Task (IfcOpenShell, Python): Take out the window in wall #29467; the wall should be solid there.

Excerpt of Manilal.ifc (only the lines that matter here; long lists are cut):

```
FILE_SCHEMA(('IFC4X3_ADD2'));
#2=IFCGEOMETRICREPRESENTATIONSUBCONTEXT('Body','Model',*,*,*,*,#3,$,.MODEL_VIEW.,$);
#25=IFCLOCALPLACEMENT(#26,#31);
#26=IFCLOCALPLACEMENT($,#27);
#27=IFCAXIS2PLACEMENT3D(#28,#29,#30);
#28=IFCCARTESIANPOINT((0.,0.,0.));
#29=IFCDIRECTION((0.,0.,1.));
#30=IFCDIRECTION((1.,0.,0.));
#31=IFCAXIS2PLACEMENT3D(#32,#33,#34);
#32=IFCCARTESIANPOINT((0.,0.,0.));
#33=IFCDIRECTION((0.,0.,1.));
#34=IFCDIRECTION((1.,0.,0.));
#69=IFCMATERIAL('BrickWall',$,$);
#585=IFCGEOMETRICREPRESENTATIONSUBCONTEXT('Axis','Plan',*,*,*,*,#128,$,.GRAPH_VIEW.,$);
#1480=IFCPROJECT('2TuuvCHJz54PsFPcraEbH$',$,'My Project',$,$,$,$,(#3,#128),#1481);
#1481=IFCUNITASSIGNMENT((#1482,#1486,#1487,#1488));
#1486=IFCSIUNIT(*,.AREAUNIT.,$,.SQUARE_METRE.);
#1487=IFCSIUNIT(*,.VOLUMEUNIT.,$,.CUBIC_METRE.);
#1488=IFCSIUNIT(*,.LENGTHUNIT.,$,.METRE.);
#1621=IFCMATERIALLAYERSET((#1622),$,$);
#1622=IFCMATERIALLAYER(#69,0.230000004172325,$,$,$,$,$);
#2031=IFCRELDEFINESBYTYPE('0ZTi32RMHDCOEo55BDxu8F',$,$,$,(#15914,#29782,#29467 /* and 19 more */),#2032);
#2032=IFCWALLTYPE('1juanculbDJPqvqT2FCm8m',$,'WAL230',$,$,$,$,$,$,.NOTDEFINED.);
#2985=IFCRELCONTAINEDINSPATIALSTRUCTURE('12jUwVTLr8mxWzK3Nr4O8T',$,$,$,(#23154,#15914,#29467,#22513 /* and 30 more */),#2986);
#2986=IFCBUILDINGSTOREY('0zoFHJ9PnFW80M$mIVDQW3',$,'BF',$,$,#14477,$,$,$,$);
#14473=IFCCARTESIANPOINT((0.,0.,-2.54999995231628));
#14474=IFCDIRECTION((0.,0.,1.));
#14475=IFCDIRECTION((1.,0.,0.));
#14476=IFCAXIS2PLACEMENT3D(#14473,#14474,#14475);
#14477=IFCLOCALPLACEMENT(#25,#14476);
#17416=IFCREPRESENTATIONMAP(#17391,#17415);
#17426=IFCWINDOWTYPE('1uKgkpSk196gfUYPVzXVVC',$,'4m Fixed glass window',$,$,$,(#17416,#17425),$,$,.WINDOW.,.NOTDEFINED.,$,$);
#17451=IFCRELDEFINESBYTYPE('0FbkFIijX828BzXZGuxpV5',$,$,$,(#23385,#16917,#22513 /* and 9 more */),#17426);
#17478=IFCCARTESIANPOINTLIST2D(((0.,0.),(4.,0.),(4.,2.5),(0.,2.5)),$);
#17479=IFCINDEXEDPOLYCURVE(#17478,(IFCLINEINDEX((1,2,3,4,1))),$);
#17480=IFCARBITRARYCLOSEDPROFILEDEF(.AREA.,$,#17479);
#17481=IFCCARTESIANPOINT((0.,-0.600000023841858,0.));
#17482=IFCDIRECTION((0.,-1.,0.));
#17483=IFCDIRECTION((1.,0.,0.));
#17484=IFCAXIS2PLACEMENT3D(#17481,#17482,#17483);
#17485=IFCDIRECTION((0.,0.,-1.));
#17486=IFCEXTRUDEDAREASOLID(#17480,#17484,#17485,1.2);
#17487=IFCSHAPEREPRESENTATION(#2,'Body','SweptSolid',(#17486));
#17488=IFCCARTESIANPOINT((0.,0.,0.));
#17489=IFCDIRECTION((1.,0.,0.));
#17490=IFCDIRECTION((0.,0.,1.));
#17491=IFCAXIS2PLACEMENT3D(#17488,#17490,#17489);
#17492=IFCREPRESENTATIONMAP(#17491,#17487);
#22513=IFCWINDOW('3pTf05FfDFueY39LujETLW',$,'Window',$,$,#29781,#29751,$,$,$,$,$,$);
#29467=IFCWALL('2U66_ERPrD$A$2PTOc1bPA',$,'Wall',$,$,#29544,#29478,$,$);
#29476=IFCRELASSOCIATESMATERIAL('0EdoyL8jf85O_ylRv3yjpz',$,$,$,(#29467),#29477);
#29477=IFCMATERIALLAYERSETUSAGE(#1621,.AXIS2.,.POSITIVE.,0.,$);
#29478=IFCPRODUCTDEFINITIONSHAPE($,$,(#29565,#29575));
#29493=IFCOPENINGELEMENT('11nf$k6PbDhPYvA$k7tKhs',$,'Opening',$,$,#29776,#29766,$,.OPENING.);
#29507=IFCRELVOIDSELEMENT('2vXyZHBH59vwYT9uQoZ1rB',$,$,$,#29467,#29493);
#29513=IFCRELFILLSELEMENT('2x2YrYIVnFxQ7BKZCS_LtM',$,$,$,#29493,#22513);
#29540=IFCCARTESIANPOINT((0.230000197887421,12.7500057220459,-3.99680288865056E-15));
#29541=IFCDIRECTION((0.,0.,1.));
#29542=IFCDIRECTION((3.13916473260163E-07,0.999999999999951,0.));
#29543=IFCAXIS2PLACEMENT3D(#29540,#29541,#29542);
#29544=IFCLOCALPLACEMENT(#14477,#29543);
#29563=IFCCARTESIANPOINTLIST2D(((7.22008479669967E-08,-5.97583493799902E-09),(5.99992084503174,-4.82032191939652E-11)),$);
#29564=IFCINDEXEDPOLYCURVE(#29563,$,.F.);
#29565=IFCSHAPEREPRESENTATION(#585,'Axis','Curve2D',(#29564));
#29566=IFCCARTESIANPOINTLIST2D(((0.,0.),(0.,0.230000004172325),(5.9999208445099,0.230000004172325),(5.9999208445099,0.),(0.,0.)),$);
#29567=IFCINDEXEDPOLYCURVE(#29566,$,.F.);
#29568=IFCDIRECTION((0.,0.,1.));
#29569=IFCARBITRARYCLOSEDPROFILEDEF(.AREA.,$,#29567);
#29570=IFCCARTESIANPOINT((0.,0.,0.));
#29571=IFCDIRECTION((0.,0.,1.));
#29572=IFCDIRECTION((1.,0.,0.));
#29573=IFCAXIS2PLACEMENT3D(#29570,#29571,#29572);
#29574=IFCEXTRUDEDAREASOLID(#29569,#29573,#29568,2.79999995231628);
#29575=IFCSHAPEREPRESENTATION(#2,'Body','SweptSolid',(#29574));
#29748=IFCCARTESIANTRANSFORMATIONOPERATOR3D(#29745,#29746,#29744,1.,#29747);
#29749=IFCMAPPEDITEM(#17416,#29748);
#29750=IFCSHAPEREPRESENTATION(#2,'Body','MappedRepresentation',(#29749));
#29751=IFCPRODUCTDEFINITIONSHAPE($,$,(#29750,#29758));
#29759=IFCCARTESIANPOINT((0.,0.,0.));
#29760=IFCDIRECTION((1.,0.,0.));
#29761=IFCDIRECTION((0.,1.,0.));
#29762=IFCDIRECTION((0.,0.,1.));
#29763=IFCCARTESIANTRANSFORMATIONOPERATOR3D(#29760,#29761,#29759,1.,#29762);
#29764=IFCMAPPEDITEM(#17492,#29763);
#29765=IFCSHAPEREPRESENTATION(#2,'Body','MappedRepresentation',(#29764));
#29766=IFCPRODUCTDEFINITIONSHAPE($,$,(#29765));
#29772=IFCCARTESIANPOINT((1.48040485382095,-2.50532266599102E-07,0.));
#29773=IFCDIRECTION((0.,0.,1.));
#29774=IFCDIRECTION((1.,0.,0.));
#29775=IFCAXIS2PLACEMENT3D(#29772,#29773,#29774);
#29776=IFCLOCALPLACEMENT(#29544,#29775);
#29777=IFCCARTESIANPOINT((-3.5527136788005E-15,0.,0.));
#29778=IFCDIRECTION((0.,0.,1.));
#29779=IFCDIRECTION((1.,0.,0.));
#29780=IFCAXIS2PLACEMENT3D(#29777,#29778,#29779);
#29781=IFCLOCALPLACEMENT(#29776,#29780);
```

```python
import ifcopenshell
import ifcopenshell.api.feature
import ifcopenshell.api.root
import ifcopenshell.geom
import ifcopenshell.util.shape

model = ifcopenshell.open("Manilal.ifc")
settings = ifcopenshell.geom.settings()


def volume(element):
    """Net volume in cubic metres, openings subtracted."""
    shape = ifcopenshell.geom.create_shape(settings, element)
    return ifcopenshell.util.shape.get_volume(shape.geometry)


window = model.by_guid("3pTf05FfDFueY39LujETLW")
opening = window.FillsVoids[0].RelatingOpeningElement
wall = opening.VoidsElements[0].RelatingBuildingElement
before = volume(wall)

ifcopenshell.api.root.remove_product(model, product=window)
ifcopenshell.api.feature.remove_feature(model, feature=opening)

after = volume(wall)

print(f"wall volume {before:.3f} -> {after:.3f} m3")

model.write("Manilal_updated.ifc")
```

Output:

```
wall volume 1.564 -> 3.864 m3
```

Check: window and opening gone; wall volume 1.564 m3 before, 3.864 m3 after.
